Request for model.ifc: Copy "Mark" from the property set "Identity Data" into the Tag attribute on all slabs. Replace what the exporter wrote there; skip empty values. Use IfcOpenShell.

First a look at what the model holds.

```python
import ifcopenshell
import ifcopenshell.util.element

model = ifcopenshell.open("model.ifc")
print(model.schema)
slabs = model.by_type("IfcSlab")
print(len(slabs), "slabs")
for e in slabs[:8]:
    source = ifcopenshell.util.element.get_pset(e, "Identity Data", "Mark")
    target = e.Tag
    print(e.id(), repr(source), repr(target), sep=" | ")
```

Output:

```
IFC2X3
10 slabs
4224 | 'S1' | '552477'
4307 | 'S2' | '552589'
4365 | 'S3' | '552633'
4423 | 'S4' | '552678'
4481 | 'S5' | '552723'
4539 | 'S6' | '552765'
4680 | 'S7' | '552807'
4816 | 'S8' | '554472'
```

```python
import ifcopenshell
import ifcopenshell.util.element

model = ifcopenshell.open("model.ifc")

count = 0
for e in model.by_type("IfcSlab"):
    value = ifcopenshell.util.element.get_pset(e, "Identity Data", "Mark")
    current = e.Tag
    if not value or not value.strip() or current == value:
        continue
    e.Tag = value
    count += 1

print(count, "slabs updated")

model.write("model-out.ifc")
```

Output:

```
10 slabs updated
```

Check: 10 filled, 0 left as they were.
